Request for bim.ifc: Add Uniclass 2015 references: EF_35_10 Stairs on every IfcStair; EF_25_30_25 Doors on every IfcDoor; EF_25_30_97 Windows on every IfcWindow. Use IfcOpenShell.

First a look at what the model holds.

```python
import ifcopenshell

model = ifcopenshell.open("bim.ifc")
print(model.schema)
print("classifications:", [c.Name for c in model.by_type("IfcClassification")])
for ifc_class in ("IfcDoor", "IfcRoof", "IfcStair", "IfcWall", "IfcWindow"):
    print(ifc_class, len(model.by_type(ifc_class)))
```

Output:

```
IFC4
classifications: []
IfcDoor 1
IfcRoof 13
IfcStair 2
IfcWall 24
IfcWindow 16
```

```python
import ifcopenshell
import ifcopenshell.api.classification

model = ifcopenshell.open("bim.ifc")

system = ifcopenshell.api.classification.add_classification(model, classification="Uniclass 2015")

codes = {
    "IfcStair": ("EF_35_10", "Stairs"),
    "IfcDoor": ("EF_25_30_25", "Doors"),
    "IfcWindow": ("EF_25_30_97", "Windows"),
}
for ifc_class, (code, name) in codes.items():
    products = model.by_type(ifc_class)
    ifcopenshell.api.classification.add_reference(
        model, products=products, classification=system, identification=code, name=name
    )
    print(code, len(products))

model.write("bim_edited.ifc")
```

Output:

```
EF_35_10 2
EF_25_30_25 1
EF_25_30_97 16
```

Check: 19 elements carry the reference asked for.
